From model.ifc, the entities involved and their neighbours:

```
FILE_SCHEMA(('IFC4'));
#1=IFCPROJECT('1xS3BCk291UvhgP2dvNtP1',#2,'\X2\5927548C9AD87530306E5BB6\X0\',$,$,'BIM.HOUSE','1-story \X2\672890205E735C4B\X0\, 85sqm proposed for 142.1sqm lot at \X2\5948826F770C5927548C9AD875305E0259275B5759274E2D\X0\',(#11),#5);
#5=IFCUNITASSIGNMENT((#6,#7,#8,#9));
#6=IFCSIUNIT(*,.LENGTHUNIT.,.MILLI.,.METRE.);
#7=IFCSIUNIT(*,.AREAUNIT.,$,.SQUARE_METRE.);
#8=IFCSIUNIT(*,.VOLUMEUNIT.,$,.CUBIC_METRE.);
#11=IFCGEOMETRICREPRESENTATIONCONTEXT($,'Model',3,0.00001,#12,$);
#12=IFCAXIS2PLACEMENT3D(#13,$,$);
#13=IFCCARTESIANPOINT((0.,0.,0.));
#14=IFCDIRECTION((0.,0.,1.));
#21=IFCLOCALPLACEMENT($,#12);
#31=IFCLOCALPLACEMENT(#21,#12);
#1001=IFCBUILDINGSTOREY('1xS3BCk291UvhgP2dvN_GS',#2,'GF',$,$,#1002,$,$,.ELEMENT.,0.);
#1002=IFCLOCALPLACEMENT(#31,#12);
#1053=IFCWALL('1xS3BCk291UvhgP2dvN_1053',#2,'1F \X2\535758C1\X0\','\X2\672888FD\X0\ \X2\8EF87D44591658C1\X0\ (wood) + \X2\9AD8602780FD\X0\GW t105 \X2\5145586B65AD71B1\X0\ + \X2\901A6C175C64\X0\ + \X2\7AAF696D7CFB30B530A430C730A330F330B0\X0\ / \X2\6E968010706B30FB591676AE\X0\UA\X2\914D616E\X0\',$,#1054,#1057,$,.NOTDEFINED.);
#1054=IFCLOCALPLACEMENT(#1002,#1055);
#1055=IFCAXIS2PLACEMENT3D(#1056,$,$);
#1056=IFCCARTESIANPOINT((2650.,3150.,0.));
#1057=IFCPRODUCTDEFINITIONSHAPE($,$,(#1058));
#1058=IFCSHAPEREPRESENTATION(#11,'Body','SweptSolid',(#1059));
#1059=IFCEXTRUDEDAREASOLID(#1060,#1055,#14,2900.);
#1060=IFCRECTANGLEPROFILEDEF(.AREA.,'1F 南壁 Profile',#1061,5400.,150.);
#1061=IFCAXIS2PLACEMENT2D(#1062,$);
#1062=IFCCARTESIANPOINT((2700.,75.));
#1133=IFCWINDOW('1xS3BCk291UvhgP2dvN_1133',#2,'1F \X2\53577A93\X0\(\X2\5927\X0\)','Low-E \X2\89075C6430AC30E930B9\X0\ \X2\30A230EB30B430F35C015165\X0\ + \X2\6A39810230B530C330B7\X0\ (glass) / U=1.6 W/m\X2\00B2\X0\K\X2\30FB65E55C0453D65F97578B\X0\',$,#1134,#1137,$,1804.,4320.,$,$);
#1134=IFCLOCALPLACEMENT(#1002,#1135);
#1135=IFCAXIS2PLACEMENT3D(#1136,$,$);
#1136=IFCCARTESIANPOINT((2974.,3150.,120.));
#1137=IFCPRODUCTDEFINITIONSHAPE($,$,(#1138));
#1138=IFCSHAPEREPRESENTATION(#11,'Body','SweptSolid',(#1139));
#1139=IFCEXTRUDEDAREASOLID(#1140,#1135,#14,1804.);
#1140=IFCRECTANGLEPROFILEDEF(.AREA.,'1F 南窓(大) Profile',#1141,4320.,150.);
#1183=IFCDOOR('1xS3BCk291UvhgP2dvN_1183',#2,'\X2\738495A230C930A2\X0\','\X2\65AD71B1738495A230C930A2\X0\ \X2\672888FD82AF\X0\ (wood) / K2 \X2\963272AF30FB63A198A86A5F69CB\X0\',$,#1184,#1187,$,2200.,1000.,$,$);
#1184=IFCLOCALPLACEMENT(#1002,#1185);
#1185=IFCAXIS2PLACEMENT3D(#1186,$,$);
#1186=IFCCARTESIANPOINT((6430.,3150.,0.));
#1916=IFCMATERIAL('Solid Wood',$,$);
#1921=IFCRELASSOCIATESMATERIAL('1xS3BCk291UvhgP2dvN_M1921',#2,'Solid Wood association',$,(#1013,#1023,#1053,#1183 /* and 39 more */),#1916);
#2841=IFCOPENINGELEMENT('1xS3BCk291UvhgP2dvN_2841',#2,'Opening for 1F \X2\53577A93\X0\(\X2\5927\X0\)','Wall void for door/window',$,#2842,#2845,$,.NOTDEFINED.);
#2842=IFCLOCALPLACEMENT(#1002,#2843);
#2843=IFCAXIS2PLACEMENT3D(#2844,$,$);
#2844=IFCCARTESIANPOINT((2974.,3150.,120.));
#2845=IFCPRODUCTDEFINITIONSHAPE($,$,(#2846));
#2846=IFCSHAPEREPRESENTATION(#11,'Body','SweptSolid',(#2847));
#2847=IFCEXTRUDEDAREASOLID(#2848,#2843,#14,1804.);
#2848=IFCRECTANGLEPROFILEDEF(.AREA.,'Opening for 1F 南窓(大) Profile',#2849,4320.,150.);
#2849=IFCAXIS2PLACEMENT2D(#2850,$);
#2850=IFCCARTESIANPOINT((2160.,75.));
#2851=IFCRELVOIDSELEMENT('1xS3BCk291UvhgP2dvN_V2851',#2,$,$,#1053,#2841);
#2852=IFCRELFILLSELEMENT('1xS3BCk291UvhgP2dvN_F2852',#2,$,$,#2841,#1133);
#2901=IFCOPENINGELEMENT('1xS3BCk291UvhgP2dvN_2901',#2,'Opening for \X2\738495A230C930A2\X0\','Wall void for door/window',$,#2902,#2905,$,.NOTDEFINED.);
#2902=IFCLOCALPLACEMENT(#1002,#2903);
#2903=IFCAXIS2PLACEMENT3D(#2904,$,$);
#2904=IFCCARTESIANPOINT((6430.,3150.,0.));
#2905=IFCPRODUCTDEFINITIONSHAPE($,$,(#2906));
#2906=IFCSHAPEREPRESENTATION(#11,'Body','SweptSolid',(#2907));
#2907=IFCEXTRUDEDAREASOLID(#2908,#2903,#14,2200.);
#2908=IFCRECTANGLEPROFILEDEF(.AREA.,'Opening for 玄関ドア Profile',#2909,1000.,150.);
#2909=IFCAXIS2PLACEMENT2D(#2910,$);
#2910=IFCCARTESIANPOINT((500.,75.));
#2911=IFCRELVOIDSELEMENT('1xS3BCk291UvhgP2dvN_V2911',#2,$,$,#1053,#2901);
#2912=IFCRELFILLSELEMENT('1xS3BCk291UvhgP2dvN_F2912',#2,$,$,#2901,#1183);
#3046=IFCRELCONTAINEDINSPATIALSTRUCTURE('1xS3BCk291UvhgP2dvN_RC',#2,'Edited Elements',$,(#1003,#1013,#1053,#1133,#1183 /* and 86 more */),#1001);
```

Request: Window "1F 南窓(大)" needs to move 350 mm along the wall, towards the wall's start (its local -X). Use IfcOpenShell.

```python
import ifcopenshell
import ifcopenshell.api.geometry
import ifcopenshell.util.placement

model = ifcopenshell.open("model.ifc")

window = model.by_guid("1xS3BCk291UvhgP2dvN_1133")
opening = window.FillsVoids[0].RelatingOpeningElement
wall = opening.VoidsElements[0].RelatingBuildingElement

wall_matrix = ifcopenshell.util.placement.get_local_placement(wall.ObjectPlacement)
shift = wall_matrix[:3, 0] * -350.0
before = ifcopenshell.util.placement.get_local_placement(window.ObjectPlacement)[:3, 3].copy()

# The window is not placed relative to its opening, so move both.
for product in (opening, window):
    matrix = ifcopenshell.util.placement.get_local_placement(product.ObjectPlacement)
    matrix[:3, 3] += shift
    ifcopenshell.api.geometry.edit_object_placement(model, product=product, matrix=matrix, is_si=False)

after = ifcopenshell.util.placement.get_local_placement(window.ObjectPlacement)[:3, 3]
print("window moved by", (after - before).round(3) + 0.0)

model.write("model_updated.ifc")
```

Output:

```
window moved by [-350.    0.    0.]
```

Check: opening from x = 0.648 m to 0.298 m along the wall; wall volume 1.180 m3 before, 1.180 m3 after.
